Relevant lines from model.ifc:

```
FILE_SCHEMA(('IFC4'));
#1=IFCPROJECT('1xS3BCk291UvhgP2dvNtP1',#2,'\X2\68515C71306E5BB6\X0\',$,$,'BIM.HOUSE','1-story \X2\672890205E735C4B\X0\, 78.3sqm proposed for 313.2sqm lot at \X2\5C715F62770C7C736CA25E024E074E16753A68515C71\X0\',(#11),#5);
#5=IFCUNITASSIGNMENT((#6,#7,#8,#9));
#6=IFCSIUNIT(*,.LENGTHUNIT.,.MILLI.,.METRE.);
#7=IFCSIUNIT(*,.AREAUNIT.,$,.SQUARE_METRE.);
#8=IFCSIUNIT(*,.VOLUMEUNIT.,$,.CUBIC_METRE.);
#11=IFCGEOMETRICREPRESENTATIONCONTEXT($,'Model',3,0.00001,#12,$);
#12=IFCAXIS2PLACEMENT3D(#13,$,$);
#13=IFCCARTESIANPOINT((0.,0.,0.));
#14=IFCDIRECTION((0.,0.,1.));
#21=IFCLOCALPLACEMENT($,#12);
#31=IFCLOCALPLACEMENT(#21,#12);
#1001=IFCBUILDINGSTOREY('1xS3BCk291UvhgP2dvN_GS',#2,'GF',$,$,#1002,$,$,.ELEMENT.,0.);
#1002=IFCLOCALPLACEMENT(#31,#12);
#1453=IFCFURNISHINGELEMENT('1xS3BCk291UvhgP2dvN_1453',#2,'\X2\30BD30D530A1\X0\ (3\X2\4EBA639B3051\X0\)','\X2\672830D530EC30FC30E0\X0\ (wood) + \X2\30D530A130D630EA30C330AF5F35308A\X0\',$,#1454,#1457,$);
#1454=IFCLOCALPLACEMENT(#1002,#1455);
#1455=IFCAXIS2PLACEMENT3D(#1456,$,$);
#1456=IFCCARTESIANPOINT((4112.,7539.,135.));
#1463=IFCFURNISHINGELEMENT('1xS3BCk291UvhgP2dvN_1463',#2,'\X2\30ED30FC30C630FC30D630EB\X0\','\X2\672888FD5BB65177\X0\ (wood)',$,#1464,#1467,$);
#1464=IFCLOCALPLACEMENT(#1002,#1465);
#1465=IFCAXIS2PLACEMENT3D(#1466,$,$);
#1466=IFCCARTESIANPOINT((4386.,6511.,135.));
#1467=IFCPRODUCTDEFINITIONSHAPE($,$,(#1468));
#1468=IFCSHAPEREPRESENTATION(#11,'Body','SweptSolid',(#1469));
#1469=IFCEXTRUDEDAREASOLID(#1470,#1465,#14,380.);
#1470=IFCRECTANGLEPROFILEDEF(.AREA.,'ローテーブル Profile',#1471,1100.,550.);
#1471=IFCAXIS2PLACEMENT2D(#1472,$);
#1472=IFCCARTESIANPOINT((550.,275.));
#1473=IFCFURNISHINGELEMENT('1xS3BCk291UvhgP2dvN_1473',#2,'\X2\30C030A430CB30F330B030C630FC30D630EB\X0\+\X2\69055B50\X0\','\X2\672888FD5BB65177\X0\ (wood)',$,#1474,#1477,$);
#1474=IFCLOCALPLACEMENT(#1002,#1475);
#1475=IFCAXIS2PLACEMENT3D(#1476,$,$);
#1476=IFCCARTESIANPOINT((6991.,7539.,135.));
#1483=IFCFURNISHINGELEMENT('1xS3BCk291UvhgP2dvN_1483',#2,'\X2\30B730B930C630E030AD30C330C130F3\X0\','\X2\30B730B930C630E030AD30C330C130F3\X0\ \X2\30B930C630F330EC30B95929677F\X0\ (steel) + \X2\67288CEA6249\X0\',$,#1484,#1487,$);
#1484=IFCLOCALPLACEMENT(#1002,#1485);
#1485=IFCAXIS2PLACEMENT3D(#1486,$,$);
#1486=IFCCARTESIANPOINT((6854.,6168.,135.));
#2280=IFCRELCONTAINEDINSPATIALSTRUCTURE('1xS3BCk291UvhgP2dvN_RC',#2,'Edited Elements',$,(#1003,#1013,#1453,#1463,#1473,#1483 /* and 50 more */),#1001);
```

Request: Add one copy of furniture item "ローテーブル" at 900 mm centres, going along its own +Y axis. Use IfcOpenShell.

```python
import ifcopenshell
import ifcopenshell.api.geometry
import ifcopenshell.api.root
import ifcopenshell.util.element
import ifcopenshell.util.placement

model = ifcopenshell.open("model.ifc")


def reuse_history(source, copy):
    """copy_class also copies each property set's owner history, people and application; keep the originals."""
    for rel in copy.IsDefinedBy:
        if rel.is_a("IfcRelDefinesByProperties") and (history := rel.RelatingPropertyDefinition.OwnerHistory):
            rel.RelatingPropertyDefinition.OwnerHistory = source.OwnerHistory
            ifcopenshell.util.element.remove_deep2(model, history)


source = model.by_guid("1xS3BCk291UvhgP2dvN_1463")
base = ifcopenshell.util.placement.get_local_placement(source.ObjectPlacement)
step = base[:3, 1] * 900.0

for i in range(1, 2):
    copy = ifcopenshell.api.root.copy_class(model, product=source)
    copy.Representation = ifcopenshell.util.element.copy_deep(
        model, source.Representation, exclude=["IfcGeometricRepresentationContext", "IfcRepresentationMap"]
    )
    reuse_history(source, copy)
    matrix = base.copy()
    matrix[:3, 3] += i * step
    print("added at", matrix[:3, 3].round(3) + 0.0)
    ifcopenshell.api.geometry.edit_object_placement(model, product=copy, matrix=matrix, is_si=False)

model.write("model-out.ifc")
```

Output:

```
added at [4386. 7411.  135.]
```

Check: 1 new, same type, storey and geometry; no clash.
